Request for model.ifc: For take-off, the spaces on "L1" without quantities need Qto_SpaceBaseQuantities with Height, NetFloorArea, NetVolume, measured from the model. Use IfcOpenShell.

First a look at what the model holds.

```python
import ifcopenshell
import ifcopenshell.util.element
import ifcopenshell.util.unit

model = ifcopenshell.open("model.ifc")
print(model.schema)
for unit_type in ("LENGTHUNIT", "AREAUNIT", "VOLUMEUNIT"):
    print(unit_type, ifcopenshell.util.unit.calculate_unit_scale(model, unit_type))
storey = next(s for s in model.by_type("IfcBuildingStorey") if s.Name == "L1")
spaces = [e for e in ifcopenshell.util.element.get_decomposition(storey) if e.is_a("IfcSpace")]
for e in sorted(spaces, key=lambda e: e.id()):
    print(e.id(), e.is_a(), e.Name, list(ifcopenshell.util.element.get_psets(e, qtos_only=True)), sep=" | ")
```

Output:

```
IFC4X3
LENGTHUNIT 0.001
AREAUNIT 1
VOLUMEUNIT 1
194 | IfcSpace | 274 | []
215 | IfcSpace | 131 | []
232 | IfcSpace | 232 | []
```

```python
import ifcopenshell
import ifcopenshell.api.pset
import ifcopenshell.geom
import ifcopenshell.util.element
import ifcopenshell.util.shape
import ifcopenshell.util.unit

model = ifcopenshell.open("model.ifc")
unit_scale = ifcopenshell.util.unit.calculate_unit_scale(model)
area_scale = ifcopenshell.util.unit.calculate_unit_scale(model, "AREAUNIT")
volume_scale = ifcopenshell.util.unit.calculate_unit_scale(model, "VOLUMEUNIT")
settings = ifcopenshell.geom.settings()

storey = next(s for s in model.by_type("IfcBuildingStorey") if s.Name == "L1")
spaces = [e for e in ifcopenshell.util.element.get_decomposition(storey) if e.is_a("IfcSpace")]

for e in sorted(spaces, key=lambda e: e.id()):
    if ifcopenshell.util.element.get_psets(e, qtos_only=True, should_inherit=False):
        continue
    # Geometry comes back in metres, in the element's own axes.
    shape = ifcopenshell.geom.create_shape(settings, e)
    values = {
        "Height": ifcopenshell.util.shape.get_z(shape.geometry) / unit_scale,
        "NetFloorArea": ifcopenshell.util.shape.get_footprint_area(shape.geometry) / area_scale,
        "NetVolume": ifcopenshell.util.shape.get_volume(shape.geometry) / volume_scale,
    }
    qto = ifcopenshell.api.pset.add_qto(model, product=e, name="Qto_SpaceBaseQuantities")
    ifcopenshell.api.pset.edit_qto(model, qto=qto, properties=values)
    print(e.id(), {k: round(v, 3) for k, v in values.items()})

model.write("model_edited.ifc")
```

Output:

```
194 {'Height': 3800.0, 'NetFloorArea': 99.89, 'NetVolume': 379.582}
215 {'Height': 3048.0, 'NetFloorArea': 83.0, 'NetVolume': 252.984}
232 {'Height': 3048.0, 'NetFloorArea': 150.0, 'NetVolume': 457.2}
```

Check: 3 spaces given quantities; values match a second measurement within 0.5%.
